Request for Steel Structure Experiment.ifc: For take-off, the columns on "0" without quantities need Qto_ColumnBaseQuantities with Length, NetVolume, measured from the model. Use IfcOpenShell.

First a look at what the model holds.

```python
import ifcopenshell
import ifcopenshell.util.element
import ifcopenshell.util.unit

model = ifcopenshell.open("Steel Structure Experiment.ifc")
print(model.schema)
for unit_type in ("LENGTHUNIT", "AREAUNIT", "VOLUMEUNIT"):
    print(unit_type, ifcopenshell.util.unit.calculate_unit_scale(model, unit_type))
storey = next(s for s in model.by_type("IfcBuildingStorey") if s.Name == "0")
columns = [e for e in ifcopenshell.util.element.get_decomposition(storey) if e.is_a("IfcColumn")]
for e in sorted(columns, key=lambda e: e.id()):
    print(e.id(), e.is_a(), e.Name, list(ifcopenshell.util.element.get_psets(e, qtos_only=True)), sep=" | ")
```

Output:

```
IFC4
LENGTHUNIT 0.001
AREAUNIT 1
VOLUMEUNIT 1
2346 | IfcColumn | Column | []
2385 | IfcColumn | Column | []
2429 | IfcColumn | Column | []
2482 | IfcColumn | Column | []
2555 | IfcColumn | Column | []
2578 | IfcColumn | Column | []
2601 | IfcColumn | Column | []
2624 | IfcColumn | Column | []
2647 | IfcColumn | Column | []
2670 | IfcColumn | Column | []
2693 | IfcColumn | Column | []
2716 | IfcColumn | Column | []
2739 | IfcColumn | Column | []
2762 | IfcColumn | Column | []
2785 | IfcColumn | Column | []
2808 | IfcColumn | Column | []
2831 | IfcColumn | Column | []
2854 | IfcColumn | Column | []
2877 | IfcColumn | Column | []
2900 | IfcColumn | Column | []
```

```python
import ifcopenshell
import ifcopenshell.api.pset
import ifcopenshell.geom
import ifcopenshell.util.element
import ifcopenshell.util.shape
import ifcopenshell.util.unit

model = ifcopenshell.open("Steel Structure Experiment.ifc")
unit_scale = ifcopenshell.util.unit.calculate_unit_scale(model)
volume_scale = ifcopenshell.util.unit.calculate_unit_scale(model, "VOLUMEUNIT")
settings = ifcopenshell.geom.settings()

storey = next(s for s in model.by_type("IfcBuildingStorey") if s.Name == "0")
columns = [e for e in ifcopenshell.util.element.get_decomposition(storey) if e.is_a("IfcColumn")]

for e in sorted(columns, key=lambda e: e.id()):
    if ifcopenshell.util.element.get_psets(e, qtos_only=True, should_inherit=False):
        continue
    # Geometry comes back in metres, in the element's own axes.
    shape = ifcopenshell.geom.create_shape(settings, e)
    values = {
        "Length": ifcopenshell.util.shape.get_z(shape.geometry) / unit_scale,
        "NetVolume": ifcopenshell.util.shape.get_volume(shape.geometry) / volume_scale,
    }
    qto = ifcopenshell.api.pset.add_qto(model, product=e, name="Qto_ColumnBaseQuantities")
    ifcopenshell.api.pset.edit_qto(model, qto=qto, properties=values)
    print(e.id(), {k: round(v, 3) for k, v in values.items()})

model.write("Steel Structure Experiment_rev.ifc")
```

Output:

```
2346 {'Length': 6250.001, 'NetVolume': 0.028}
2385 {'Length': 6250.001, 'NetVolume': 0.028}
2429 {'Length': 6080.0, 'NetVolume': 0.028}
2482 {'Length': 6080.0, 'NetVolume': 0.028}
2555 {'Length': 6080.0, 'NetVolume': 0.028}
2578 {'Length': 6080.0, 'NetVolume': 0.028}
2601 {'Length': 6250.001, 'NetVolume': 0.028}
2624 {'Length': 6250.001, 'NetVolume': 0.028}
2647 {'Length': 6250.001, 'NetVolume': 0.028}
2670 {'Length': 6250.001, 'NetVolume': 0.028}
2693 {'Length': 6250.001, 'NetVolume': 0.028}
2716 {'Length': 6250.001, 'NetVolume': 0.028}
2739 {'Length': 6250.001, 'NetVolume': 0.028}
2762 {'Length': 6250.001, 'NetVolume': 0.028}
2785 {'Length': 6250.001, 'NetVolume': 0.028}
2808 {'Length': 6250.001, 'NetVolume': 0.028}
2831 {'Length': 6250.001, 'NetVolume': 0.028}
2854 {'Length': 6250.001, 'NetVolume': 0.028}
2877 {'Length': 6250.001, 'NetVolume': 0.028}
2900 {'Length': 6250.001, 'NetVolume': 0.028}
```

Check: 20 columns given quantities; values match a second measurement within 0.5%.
